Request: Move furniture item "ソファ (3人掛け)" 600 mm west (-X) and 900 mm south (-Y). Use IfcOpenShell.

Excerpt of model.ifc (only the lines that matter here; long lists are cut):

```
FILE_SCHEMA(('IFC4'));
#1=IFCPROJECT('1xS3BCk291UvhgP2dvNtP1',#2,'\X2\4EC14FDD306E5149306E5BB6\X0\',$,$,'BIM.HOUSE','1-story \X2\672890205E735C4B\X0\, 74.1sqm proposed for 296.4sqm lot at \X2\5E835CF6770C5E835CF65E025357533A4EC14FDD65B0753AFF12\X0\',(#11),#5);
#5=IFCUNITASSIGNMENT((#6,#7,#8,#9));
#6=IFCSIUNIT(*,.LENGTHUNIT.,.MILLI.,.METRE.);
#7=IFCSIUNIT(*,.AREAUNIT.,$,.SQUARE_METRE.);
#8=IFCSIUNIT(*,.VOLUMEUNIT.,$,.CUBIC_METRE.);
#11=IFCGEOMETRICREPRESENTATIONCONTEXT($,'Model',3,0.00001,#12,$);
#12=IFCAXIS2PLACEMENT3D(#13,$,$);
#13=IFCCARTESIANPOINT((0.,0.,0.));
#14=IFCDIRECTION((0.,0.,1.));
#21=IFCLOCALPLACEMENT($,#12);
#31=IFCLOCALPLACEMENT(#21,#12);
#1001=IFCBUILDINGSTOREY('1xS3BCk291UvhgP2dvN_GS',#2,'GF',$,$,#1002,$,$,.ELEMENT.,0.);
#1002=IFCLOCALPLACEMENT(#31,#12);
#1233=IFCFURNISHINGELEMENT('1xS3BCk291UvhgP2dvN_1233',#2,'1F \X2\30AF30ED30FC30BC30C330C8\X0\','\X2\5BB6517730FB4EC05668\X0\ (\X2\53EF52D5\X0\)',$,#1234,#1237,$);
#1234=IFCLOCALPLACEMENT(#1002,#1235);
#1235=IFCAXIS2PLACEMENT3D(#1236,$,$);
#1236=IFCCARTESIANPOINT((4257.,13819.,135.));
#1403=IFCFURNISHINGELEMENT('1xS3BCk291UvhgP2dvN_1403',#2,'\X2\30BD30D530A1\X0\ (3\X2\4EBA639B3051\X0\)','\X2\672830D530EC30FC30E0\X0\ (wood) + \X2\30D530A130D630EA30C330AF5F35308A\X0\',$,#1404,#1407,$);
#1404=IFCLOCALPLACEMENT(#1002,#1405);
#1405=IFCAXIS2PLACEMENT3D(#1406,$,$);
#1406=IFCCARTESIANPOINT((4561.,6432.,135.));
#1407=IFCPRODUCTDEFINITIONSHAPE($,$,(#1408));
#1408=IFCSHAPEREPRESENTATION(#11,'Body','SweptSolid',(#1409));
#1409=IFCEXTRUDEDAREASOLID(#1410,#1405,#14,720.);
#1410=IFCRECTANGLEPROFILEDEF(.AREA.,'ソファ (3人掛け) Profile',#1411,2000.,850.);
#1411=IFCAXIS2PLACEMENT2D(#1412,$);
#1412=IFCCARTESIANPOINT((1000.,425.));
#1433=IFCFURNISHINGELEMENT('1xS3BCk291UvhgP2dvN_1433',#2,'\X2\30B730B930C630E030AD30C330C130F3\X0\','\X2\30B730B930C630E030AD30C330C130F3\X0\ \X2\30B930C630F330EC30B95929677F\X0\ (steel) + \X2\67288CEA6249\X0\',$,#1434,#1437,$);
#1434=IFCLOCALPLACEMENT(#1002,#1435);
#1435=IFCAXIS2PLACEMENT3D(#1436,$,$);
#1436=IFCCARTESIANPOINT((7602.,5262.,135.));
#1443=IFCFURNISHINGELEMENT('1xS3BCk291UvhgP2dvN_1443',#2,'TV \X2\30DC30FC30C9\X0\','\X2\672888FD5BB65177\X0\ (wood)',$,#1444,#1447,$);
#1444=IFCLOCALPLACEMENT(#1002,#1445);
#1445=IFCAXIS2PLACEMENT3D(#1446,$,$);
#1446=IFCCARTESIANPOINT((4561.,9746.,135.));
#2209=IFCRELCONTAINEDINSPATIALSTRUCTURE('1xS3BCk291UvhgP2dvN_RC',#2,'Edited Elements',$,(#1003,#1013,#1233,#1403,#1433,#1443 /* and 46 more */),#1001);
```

```python
import ifcopenshell
import ifcopenshell.api.geometry
import ifcopenshell.util.placement
import ifcopenshell.util.unit

model = ifcopenshell.open("model.ifc")
unit_scale = ifcopenshell.util.unit.calculate_unit_scale(model)

item = model.by_id(1403)
matrix = ifcopenshell.util.placement.get_local_placement(item.ObjectPlacement)
matrix[0, 3] -= 0.6 / unit_scale
matrix[1, 3] -= 0.9 / unit_scale
ifcopenshell.api.geometry.edit_object_placement(model, product=item, matrix=matrix, is_si=False)

print(ifcopenshell.util.placement.get_local_placement(item.ObjectPlacement).round(3) + 0.0)

model.write("model_edited.ifc")
```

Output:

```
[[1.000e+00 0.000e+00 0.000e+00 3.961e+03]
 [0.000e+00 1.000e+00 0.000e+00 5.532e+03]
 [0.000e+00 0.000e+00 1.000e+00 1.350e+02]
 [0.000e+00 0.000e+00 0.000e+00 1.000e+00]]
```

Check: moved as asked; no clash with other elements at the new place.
